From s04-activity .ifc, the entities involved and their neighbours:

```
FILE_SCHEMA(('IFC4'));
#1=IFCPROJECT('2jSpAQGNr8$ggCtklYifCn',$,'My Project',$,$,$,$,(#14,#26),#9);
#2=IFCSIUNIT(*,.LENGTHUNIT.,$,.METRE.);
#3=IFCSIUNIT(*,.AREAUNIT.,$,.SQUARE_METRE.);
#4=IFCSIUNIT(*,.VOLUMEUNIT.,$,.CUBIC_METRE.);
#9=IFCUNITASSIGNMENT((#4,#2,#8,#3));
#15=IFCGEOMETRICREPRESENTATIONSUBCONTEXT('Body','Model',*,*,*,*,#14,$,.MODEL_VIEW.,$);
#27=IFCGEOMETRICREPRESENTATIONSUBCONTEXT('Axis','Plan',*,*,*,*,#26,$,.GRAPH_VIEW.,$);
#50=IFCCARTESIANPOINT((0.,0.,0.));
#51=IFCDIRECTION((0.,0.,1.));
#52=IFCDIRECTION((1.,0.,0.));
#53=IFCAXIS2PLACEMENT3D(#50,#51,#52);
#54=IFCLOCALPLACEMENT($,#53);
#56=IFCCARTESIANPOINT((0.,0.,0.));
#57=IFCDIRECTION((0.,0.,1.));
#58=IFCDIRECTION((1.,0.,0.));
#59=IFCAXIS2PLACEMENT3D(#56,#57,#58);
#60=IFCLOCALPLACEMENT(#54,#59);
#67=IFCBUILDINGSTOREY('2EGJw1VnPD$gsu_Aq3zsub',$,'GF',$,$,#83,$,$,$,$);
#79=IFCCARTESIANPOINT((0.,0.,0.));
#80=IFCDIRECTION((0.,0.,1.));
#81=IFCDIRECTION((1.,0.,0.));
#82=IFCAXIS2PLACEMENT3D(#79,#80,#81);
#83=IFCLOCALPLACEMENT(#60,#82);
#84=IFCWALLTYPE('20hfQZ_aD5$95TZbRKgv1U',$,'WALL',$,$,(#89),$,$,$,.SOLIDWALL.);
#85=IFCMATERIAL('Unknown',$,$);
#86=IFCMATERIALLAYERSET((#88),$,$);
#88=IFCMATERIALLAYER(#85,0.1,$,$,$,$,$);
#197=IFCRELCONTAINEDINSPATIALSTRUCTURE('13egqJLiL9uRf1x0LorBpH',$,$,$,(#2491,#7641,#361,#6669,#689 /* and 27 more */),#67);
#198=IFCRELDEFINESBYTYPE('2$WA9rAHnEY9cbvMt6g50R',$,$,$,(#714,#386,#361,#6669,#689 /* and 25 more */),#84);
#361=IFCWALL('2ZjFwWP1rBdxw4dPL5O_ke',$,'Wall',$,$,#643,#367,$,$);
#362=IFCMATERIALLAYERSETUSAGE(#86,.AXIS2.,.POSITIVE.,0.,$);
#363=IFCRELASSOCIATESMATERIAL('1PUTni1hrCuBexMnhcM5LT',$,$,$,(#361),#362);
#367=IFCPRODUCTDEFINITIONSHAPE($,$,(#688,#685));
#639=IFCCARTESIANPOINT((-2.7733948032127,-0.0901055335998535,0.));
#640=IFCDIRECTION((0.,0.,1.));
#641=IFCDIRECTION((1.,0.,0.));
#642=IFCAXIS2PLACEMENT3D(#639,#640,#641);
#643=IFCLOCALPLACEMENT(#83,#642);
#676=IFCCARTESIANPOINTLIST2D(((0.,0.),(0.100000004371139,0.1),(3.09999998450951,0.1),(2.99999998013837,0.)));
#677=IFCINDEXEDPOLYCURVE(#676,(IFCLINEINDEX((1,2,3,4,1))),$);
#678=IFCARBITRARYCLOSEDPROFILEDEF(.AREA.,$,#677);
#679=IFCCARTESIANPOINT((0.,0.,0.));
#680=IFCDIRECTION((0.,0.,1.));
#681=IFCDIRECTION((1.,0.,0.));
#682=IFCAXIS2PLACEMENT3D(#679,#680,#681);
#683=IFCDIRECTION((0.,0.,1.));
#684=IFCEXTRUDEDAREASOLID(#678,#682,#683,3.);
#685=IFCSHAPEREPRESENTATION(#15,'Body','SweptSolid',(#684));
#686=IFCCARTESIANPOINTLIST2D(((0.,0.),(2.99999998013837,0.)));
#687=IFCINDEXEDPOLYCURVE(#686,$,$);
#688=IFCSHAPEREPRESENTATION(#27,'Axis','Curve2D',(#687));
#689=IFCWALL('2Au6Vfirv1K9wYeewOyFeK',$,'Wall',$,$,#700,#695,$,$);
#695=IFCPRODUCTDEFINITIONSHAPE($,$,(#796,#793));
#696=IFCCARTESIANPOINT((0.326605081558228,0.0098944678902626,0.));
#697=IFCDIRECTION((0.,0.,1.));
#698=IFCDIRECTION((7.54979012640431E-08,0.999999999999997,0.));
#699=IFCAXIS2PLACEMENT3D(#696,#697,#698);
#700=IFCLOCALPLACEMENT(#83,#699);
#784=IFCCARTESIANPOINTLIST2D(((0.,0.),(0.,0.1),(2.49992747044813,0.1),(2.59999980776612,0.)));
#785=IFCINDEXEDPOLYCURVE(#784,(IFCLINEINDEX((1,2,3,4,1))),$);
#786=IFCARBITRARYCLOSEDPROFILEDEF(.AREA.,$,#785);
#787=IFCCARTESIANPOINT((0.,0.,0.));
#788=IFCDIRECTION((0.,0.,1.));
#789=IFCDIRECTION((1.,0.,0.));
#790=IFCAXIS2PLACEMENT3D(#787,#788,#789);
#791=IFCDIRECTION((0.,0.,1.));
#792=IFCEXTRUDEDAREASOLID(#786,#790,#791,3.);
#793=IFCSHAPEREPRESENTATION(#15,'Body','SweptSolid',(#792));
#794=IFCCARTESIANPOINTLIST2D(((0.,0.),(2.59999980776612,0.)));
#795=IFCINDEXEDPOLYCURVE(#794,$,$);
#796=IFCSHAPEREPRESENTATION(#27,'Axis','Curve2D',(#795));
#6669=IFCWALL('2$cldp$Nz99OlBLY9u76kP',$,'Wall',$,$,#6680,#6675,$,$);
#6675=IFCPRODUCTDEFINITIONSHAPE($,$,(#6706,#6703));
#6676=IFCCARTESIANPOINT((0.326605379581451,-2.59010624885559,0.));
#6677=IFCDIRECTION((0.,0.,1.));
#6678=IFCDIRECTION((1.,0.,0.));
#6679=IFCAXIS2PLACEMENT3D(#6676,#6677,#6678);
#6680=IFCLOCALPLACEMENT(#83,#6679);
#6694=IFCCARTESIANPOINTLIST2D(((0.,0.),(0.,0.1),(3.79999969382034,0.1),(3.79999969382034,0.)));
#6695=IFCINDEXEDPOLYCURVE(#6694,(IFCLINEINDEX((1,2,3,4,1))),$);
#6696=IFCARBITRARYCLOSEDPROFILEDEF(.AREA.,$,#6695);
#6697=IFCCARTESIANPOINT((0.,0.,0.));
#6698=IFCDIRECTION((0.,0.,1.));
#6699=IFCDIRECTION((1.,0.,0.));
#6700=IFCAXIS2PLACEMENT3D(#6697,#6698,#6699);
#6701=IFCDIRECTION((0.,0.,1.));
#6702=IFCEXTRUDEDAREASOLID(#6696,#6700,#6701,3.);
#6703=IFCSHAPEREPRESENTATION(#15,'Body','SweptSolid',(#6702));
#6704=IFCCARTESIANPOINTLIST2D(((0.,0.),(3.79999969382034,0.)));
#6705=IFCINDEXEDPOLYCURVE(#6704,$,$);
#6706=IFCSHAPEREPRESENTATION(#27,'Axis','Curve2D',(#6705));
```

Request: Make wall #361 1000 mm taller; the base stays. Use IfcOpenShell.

```python
import ifcopenshell
import ifcopenshell.geom
import ifcopenshell.util.representation
import ifcopenshell.util.shape
import ifcopenshell.util.unit

model = ifcopenshell.open("s04-activity .ifc")
unit_scale = ifcopenshell.util.unit.calculate_unit_scale(model)
settings = ifcopenshell.geom.settings()


def volume(element):
    """Net volume in cubic metres, openings subtracted."""
    shape = ifcopenshell.geom.create_shape(settings, element)
    return ifcopenshell.util.shape.get_volume(shape.geometry)


wall = model.by_id(361)
before = volume(wall)

body = ifcopenshell.util.representation.get_representation(wall, "Model", "Body")
solid = body.Items[0]
old_height = solid.Depth
solid.Depth += 1 / unit_scale
after = volume(wall)

print(f"height {old_height:g} -> {solid.Depth:g}, volume {before:.3f} -> {after:.3f} m3")

model.write("s04-activity _edited.ifc")
```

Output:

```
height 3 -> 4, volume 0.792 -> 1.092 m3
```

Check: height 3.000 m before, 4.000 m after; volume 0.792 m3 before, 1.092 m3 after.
